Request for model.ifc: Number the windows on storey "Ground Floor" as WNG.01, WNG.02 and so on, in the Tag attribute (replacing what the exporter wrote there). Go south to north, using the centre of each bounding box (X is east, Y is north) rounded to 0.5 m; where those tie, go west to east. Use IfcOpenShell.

First a look at what the model holds.

```python
import ifcopenshell
import ifcopenshell.util.element
import ifcopenshell.util.placement

model = ifcopenshell.open("model.ifc")
print(model.schema)
storey = next(s for s in model.by_type("IfcBuildingStorey") if s.Name == "Ground Floor")
windows = [e for e in ifcopenshell.util.element.get_decomposition(storey) if e.is_a("IfcWindow")]
for e in sorted(windows, key=lambda e: e.id()):
    origin = ifcopenshell.util.placement.get_local_placement(e.ObjectPlacement)[:3, 3]
    print(e.id(), e.Tag, e.Name, origin.round(2) + 0.0, sep=" | ")
```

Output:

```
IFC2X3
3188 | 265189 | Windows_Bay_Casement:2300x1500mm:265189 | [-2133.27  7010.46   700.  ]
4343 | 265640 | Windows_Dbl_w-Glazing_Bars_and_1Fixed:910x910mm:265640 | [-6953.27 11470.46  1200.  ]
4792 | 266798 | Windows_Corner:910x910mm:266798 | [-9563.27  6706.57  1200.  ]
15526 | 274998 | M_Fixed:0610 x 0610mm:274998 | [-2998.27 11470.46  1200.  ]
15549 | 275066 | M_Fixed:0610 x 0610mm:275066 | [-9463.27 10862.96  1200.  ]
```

```python
import ifcopenshell
import ifcopenshell.geom
import ifcopenshell.util.element
import ifcopenshell.util.shape

model = ifcopenshell.open("model.ifc")
settings = ifcopenshell.geom.settings()
settings.set("use-world-coords", True)


def centre(element):
    shape = ifcopenshell.geom.create_shape(settings, element)
    return ifcopenshell.util.shape.get_bbox_centroid(shape.geometry)


storey = next(s for s in model.by_type("IfcBuildingStorey") if s.Name == "Ground Floor")
windows = [e for e in ifcopenshell.util.element.get_decomposition(storey) if e.is_a("IfcWindow")]

# Insertion points can sit at a corner or the storey origin, so sort by the geometry (in metres).
centres = {e: centre(e) for e in windows}
windows.sort(key=lambda e: (round(centres[e][1] / 0.5), centres[e][0]))

for i, e in enumerate(windows, start=1):
    number = f"WNG.{i:02d}"
    e.Tag = number
    print(e.id(), number)

model.write("model_updated.ifc")
```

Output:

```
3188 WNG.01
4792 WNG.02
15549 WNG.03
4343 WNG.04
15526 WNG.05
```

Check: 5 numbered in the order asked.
